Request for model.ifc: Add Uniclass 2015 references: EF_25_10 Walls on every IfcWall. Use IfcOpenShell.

First a look at what the model holds.

```python
import ifcopenshell

model = ifcopenshell.open("model.ifc")
print(model.schema)
print("classifications:", [c.Name for c in model.by_type("IfcClassification")])
for ifc_class in ("IfcDoor", "IfcRoof", "IfcStair", "IfcWall", "IfcWindow"):
    print(ifc_class, len(model.by_type(ifc_class)))
```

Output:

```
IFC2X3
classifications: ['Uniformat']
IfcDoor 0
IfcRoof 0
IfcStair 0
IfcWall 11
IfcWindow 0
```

```python
import ifcopenshell
import ifcopenshell.api.classification

model = ifcopenshell.open("model.ifc")

# IFC2X3 requires Source and Edition and has no link from the project to the system.
system = model.create_entity("IfcClassification", Source="NBS", Edition="2015", Name="Uniclass 2015")

codes = {
    "IfcWall": ("EF_25_10", "Walls"),
}
for ifc_class, (code, name) in codes.items():
    products = model.by_type(ifc_class)
    ifcopenshell.api.classification.add_reference(
        model, products=products, classification=system, identification=code, name=name
    )
    print(code, len(products))

model.write("model_v2.ifc")
```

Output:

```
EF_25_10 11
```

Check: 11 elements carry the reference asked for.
